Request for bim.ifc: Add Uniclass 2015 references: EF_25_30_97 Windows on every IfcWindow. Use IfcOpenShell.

First a look at what the model holds.

```python
import ifcopenshell

model = ifcopenshell.open("bim.ifc")
print(model.schema)
print("classifications:", [c.Name for c in model.by_type("IfcClassification")])
for ifc_class in ("IfcDoor", "IfcRoof", "IfcStair", "IfcWall", "IfcWindow"):
    print(ifc_class, len(model.by_type(ifc_class)))
```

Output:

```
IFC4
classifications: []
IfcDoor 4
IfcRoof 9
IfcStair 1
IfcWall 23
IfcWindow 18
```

```python
import ifcopenshell
import ifcopenshell.api.classification

model = ifcopenshell.open("bim.ifc")

system = ifcopenshell.api.classification.add_classification(model, classification="Uniclass 2015")

codes = {
    "IfcWindow": ("EF_25_30_97", "Windows"),
}
for ifc_class, (code, name) in codes.items():
    products = model.by_type(ifc_class)
    ifcopenshell.api.classification.add_reference(
        model, products=products, classification=system, identification=code, name=name
    )
    print(code, len(products))

model.write("bim_edited.ifc")
```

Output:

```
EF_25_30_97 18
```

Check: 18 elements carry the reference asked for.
